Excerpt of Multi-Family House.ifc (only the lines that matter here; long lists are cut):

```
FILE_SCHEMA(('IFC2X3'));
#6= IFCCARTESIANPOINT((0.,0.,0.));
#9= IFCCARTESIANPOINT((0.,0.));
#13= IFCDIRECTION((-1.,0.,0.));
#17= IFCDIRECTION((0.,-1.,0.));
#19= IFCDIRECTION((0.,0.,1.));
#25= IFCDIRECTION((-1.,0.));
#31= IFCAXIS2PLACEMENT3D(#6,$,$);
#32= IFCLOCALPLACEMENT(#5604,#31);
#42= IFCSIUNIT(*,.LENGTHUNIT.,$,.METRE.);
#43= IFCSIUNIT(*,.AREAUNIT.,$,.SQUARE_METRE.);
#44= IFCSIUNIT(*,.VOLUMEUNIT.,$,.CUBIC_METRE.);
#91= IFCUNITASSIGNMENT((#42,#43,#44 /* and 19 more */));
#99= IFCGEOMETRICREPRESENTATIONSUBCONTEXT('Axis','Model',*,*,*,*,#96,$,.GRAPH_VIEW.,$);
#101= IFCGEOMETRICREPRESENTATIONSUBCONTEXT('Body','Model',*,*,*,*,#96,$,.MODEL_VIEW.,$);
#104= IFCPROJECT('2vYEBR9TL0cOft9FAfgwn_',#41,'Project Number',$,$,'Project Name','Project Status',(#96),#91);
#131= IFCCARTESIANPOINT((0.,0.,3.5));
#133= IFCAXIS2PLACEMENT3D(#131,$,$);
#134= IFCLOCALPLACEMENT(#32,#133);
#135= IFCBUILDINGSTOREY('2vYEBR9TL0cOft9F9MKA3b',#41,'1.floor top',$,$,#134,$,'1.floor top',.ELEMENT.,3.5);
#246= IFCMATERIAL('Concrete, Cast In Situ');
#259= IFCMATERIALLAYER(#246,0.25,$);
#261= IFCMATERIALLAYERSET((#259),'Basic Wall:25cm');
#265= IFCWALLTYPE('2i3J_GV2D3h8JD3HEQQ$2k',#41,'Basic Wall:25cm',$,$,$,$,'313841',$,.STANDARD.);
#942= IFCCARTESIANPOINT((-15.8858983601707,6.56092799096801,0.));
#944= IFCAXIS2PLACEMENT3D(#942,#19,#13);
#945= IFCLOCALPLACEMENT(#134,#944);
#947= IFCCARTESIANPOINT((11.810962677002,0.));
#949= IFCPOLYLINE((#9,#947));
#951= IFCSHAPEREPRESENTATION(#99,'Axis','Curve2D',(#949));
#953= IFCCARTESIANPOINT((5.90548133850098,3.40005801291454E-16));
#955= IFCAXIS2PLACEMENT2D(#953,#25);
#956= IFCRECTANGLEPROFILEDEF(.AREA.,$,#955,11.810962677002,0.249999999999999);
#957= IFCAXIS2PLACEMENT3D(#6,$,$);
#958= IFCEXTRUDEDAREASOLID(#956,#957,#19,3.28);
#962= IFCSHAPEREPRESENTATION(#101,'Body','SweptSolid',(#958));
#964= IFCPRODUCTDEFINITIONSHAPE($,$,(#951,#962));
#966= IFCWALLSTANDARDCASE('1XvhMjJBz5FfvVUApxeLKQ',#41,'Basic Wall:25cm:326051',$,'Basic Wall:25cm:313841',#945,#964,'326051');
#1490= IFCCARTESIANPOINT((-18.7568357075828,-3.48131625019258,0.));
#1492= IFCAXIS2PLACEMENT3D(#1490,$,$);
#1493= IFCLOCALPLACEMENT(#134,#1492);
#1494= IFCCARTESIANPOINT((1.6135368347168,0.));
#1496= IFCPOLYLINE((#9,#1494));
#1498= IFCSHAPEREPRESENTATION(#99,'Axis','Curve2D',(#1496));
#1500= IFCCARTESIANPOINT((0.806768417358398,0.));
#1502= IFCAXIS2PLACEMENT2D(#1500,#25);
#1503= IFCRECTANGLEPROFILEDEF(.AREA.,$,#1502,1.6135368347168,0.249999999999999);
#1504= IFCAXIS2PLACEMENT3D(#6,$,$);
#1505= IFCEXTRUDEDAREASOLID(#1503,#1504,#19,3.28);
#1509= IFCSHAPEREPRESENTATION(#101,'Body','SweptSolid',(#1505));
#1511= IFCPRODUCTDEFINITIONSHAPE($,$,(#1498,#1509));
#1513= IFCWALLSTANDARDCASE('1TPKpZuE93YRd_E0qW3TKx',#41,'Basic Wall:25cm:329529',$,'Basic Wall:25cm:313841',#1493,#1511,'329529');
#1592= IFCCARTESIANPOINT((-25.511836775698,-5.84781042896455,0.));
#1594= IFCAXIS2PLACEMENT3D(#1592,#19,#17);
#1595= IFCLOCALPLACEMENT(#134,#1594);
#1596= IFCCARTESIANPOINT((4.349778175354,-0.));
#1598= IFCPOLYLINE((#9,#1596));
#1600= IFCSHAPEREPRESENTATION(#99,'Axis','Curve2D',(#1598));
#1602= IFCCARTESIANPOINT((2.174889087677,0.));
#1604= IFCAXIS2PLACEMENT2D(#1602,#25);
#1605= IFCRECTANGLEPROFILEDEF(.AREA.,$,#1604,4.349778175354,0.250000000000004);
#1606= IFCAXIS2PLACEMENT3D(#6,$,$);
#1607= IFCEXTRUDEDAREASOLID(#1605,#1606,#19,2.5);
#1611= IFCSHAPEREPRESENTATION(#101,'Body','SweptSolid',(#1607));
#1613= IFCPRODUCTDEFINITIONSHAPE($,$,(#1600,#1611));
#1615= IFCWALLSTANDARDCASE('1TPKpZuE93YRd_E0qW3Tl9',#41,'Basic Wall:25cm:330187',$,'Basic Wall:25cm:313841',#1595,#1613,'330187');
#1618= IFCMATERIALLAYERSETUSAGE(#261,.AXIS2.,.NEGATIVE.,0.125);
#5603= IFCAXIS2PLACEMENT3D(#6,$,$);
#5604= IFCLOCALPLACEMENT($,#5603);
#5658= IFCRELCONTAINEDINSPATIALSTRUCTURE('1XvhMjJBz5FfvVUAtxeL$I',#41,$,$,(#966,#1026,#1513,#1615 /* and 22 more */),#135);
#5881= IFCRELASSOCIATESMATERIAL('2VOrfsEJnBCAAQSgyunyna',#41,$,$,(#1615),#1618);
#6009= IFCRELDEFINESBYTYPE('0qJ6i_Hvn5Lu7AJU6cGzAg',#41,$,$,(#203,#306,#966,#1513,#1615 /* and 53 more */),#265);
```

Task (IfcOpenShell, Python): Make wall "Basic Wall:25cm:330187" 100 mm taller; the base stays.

```python
import ifcopenshell
import ifcopenshell.geom
import ifcopenshell.util.representation
import ifcopenshell.util.shape
import ifcopenshell.util.unit

model = ifcopenshell.open("Multi-Family House.ifc")
unit_scale = ifcopenshell.util.unit.calculate_unit_scale(model)
settings = ifcopenshell.geom.settings()


def volume(element):
    """Net volume in cubic metres, openings subtracted."""
    shape = ifcopenshell.geom.create_shape(settings, element)
    return ifcopenshell.util.shape.get_volume(shape.geometry)


wall = model.by_guid("1TPKpZuE93YRd_E0qW3Tl9")
before = volume(wall)

body = ifcopenshell.util.representation.get_representation(wall, "Model", "Body")
solid = body.Items[0]
old_height = solid.Depth
solid.Depth += 0.1 / unit_scale
after = volume(wall)

print(f"height {old_height:g} -> {solid.Depth:g}, volume {before:.3f} -> {after:.3f} m3")

model.write("Multi-Family House_rev.ifc")
```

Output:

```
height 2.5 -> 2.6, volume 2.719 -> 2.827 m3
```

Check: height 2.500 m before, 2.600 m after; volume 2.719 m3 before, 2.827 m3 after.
